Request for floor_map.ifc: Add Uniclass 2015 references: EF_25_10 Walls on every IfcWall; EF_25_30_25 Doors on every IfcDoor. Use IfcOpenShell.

First a look at what the model holds.

```python
import ifcopenshell

model = ifcopenshell.open("floor_map.ifc")
print(model.schema)
print("classifications:", [c.Name for c in model.by_type("IfcClassification")])
for ifc_class in ("IfcDoor", "IfcRoof", "IfcStair", "IfcWall", "IfcWindow"):
    print(ifc_class, len(model.by_type(ifc_class)))
```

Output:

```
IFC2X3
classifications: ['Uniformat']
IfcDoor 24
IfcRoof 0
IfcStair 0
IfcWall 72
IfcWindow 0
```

```python
import ifcopenshell
import ifcopenshell.api.classification

model = ifcopenshell.open("floor_map.ifc")

# IFC2X3 requires Source and Edition and has no link from the project to the system.
system = model.create_entity("IfcClassification", Source="NBS", Edition="2015", Name="Uniclass 2015")

codes = {
    "IfcWall": ("EF_25_10", "Walls"),
    "IfcDoor": ("EF_25_30_25", "Doors"),
}
for ifc_class, (code, name) in codes.items():
    products = model.by_type(ifc_class)
    ifcopenshell.api.classification.add_reference(
        model, products=products, classification=system, identification=code, name=name
    )
    print(code, len(products))

model.write("floor_map_v2.ifc")
```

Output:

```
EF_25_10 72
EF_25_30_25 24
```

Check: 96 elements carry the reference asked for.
